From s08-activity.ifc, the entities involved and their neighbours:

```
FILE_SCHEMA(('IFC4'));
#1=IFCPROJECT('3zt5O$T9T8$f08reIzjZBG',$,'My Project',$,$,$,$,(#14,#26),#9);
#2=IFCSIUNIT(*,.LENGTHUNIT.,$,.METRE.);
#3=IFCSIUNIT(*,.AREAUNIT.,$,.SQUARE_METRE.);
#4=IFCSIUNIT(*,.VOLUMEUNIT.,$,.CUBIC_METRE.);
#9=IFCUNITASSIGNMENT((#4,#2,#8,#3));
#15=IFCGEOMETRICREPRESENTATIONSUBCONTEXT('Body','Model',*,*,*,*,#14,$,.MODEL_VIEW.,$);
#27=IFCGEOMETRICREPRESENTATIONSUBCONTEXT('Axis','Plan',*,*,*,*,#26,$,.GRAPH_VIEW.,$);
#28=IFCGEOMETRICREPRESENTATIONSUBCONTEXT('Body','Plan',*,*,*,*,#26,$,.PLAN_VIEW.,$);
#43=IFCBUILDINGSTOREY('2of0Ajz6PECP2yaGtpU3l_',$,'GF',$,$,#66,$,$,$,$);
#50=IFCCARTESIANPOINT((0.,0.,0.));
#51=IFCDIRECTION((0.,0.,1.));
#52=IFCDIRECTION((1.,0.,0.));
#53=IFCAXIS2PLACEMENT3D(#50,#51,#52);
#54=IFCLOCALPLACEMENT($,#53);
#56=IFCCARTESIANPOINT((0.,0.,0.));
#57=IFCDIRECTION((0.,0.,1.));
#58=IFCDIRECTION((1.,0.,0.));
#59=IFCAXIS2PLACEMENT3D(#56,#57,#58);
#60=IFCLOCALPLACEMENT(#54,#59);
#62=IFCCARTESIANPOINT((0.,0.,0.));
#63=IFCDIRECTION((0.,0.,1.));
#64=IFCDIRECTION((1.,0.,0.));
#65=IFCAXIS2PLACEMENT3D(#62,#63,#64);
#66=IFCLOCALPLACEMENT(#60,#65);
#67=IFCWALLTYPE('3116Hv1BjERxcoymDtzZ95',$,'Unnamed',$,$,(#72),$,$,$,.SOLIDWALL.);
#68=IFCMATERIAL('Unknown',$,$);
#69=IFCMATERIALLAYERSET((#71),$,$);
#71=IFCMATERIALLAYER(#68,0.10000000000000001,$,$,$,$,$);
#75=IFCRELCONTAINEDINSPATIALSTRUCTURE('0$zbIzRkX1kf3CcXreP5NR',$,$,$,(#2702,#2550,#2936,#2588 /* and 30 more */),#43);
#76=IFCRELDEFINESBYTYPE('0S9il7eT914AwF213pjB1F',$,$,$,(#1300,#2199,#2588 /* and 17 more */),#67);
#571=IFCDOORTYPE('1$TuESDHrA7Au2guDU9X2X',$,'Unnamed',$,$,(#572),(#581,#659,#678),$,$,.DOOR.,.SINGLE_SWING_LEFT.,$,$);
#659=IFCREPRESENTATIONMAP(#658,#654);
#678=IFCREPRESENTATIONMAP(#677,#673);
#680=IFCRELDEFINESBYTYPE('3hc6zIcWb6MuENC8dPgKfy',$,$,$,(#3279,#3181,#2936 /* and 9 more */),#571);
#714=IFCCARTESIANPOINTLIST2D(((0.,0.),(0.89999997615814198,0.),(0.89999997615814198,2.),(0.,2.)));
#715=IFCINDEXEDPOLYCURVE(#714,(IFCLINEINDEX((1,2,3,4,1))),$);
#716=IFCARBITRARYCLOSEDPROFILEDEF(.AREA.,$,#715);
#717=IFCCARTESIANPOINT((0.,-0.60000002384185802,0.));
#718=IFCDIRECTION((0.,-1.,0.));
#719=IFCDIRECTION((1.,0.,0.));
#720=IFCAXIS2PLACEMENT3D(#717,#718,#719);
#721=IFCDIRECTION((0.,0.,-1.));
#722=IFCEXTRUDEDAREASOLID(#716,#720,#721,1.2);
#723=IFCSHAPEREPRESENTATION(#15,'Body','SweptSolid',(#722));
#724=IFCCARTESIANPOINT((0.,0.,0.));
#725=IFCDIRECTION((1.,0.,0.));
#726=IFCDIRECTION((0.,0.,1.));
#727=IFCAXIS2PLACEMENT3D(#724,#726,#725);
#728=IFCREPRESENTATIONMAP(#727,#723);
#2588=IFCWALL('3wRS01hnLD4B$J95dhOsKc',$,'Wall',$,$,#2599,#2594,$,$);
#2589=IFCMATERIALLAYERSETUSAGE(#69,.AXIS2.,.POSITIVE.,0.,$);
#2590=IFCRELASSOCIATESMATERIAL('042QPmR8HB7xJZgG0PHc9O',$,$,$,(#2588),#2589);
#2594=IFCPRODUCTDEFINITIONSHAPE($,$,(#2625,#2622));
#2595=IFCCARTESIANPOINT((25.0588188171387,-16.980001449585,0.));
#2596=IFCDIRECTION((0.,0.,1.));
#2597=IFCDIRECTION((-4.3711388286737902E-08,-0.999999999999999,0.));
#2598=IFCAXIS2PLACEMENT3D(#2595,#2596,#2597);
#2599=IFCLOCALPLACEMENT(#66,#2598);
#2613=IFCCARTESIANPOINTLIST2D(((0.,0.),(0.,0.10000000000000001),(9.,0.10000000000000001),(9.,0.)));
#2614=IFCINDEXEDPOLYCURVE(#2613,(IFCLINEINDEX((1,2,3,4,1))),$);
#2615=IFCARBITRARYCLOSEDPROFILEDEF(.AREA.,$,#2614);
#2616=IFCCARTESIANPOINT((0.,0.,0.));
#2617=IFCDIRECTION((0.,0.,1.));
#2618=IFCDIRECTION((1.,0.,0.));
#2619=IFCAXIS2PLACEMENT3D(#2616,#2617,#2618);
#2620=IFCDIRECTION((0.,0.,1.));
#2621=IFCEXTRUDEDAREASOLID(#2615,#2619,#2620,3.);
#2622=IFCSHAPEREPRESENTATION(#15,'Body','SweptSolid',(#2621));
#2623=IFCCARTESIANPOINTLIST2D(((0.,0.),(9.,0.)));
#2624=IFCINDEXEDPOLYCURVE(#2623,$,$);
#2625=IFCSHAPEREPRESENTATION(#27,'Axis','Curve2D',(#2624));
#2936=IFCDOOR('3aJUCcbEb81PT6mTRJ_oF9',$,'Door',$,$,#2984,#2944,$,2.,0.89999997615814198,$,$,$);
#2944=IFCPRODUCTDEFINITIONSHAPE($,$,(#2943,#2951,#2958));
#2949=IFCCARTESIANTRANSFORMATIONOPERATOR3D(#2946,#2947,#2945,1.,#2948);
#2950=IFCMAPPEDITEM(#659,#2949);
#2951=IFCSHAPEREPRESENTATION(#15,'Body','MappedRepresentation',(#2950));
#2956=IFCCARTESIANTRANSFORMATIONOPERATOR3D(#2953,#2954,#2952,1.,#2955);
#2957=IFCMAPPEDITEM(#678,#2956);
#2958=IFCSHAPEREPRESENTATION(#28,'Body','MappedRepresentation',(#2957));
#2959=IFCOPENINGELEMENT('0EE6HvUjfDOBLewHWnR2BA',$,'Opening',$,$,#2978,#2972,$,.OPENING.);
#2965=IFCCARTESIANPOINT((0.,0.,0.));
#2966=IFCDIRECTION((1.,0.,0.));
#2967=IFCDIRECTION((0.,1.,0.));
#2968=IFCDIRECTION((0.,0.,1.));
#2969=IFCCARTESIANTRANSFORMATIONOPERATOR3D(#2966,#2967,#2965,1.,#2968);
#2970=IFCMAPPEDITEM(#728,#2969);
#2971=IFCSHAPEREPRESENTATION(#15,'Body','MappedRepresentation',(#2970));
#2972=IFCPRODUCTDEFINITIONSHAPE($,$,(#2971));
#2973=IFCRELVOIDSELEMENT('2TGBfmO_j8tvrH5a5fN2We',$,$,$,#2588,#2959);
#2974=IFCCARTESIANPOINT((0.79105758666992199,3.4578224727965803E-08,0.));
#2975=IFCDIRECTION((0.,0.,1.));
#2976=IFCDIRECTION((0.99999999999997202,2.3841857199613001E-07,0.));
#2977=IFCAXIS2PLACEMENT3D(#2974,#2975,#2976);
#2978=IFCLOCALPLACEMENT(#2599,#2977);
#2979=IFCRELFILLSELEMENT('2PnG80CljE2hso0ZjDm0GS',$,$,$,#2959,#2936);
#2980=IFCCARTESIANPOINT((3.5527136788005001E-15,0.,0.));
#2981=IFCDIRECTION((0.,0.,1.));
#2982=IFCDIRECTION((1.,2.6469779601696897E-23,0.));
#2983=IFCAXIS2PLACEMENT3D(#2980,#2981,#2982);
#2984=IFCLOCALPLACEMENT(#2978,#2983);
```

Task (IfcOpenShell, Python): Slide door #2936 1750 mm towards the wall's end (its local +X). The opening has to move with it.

```python
import ifcopenshell
import ifcopenshell.api.geometry
import ifcopenshell.util.placement
import ifcopenshell.util.unit

model = ifcopenshell.open("s08-activity.ifc")
unit_scale = ifcopenshell.util.unit.calculate_unit_scale(model)

door = model.by_guid("3aJUCcbEb81PT6mTRJ_oF9")
opening = door.FillsVoids[0].RelatingOpeningElement
wall = opening.VoidsElements[0].RelatingBuildingElement

wall_matrix = ifcopenshell.util.placement.get_local_placement(wall.ObjectPlacement)
shift = wall_matrix[:3, 0] * 1.75 / unit_scale
before = ifcopenshell.util.placement.get_local_placement(door.ObjectPlacement)[:3, 3].copy()

# The door is placed relative to its opening, so it follows when the opening moves.
matrix = ifcopenshell.util.placement.get_local_placement(opening.ObjectPlacement)
matrix[:3, 3] += shift
ifcopenshell.api.geometry.edit_object_placement(
    model, product=opening, matrix=matrix, is_si=False, should_transform_children=True
)

after = ifcopenshell.util.placement.get_local_placement(door.ObjectPlacement)[:3, 3]
print("door moved by", (after - before).round(3) + 0.0)

model.write("s08-activity_rev.ifc")
```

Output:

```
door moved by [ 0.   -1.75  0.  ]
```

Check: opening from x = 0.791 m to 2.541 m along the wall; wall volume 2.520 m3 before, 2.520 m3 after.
